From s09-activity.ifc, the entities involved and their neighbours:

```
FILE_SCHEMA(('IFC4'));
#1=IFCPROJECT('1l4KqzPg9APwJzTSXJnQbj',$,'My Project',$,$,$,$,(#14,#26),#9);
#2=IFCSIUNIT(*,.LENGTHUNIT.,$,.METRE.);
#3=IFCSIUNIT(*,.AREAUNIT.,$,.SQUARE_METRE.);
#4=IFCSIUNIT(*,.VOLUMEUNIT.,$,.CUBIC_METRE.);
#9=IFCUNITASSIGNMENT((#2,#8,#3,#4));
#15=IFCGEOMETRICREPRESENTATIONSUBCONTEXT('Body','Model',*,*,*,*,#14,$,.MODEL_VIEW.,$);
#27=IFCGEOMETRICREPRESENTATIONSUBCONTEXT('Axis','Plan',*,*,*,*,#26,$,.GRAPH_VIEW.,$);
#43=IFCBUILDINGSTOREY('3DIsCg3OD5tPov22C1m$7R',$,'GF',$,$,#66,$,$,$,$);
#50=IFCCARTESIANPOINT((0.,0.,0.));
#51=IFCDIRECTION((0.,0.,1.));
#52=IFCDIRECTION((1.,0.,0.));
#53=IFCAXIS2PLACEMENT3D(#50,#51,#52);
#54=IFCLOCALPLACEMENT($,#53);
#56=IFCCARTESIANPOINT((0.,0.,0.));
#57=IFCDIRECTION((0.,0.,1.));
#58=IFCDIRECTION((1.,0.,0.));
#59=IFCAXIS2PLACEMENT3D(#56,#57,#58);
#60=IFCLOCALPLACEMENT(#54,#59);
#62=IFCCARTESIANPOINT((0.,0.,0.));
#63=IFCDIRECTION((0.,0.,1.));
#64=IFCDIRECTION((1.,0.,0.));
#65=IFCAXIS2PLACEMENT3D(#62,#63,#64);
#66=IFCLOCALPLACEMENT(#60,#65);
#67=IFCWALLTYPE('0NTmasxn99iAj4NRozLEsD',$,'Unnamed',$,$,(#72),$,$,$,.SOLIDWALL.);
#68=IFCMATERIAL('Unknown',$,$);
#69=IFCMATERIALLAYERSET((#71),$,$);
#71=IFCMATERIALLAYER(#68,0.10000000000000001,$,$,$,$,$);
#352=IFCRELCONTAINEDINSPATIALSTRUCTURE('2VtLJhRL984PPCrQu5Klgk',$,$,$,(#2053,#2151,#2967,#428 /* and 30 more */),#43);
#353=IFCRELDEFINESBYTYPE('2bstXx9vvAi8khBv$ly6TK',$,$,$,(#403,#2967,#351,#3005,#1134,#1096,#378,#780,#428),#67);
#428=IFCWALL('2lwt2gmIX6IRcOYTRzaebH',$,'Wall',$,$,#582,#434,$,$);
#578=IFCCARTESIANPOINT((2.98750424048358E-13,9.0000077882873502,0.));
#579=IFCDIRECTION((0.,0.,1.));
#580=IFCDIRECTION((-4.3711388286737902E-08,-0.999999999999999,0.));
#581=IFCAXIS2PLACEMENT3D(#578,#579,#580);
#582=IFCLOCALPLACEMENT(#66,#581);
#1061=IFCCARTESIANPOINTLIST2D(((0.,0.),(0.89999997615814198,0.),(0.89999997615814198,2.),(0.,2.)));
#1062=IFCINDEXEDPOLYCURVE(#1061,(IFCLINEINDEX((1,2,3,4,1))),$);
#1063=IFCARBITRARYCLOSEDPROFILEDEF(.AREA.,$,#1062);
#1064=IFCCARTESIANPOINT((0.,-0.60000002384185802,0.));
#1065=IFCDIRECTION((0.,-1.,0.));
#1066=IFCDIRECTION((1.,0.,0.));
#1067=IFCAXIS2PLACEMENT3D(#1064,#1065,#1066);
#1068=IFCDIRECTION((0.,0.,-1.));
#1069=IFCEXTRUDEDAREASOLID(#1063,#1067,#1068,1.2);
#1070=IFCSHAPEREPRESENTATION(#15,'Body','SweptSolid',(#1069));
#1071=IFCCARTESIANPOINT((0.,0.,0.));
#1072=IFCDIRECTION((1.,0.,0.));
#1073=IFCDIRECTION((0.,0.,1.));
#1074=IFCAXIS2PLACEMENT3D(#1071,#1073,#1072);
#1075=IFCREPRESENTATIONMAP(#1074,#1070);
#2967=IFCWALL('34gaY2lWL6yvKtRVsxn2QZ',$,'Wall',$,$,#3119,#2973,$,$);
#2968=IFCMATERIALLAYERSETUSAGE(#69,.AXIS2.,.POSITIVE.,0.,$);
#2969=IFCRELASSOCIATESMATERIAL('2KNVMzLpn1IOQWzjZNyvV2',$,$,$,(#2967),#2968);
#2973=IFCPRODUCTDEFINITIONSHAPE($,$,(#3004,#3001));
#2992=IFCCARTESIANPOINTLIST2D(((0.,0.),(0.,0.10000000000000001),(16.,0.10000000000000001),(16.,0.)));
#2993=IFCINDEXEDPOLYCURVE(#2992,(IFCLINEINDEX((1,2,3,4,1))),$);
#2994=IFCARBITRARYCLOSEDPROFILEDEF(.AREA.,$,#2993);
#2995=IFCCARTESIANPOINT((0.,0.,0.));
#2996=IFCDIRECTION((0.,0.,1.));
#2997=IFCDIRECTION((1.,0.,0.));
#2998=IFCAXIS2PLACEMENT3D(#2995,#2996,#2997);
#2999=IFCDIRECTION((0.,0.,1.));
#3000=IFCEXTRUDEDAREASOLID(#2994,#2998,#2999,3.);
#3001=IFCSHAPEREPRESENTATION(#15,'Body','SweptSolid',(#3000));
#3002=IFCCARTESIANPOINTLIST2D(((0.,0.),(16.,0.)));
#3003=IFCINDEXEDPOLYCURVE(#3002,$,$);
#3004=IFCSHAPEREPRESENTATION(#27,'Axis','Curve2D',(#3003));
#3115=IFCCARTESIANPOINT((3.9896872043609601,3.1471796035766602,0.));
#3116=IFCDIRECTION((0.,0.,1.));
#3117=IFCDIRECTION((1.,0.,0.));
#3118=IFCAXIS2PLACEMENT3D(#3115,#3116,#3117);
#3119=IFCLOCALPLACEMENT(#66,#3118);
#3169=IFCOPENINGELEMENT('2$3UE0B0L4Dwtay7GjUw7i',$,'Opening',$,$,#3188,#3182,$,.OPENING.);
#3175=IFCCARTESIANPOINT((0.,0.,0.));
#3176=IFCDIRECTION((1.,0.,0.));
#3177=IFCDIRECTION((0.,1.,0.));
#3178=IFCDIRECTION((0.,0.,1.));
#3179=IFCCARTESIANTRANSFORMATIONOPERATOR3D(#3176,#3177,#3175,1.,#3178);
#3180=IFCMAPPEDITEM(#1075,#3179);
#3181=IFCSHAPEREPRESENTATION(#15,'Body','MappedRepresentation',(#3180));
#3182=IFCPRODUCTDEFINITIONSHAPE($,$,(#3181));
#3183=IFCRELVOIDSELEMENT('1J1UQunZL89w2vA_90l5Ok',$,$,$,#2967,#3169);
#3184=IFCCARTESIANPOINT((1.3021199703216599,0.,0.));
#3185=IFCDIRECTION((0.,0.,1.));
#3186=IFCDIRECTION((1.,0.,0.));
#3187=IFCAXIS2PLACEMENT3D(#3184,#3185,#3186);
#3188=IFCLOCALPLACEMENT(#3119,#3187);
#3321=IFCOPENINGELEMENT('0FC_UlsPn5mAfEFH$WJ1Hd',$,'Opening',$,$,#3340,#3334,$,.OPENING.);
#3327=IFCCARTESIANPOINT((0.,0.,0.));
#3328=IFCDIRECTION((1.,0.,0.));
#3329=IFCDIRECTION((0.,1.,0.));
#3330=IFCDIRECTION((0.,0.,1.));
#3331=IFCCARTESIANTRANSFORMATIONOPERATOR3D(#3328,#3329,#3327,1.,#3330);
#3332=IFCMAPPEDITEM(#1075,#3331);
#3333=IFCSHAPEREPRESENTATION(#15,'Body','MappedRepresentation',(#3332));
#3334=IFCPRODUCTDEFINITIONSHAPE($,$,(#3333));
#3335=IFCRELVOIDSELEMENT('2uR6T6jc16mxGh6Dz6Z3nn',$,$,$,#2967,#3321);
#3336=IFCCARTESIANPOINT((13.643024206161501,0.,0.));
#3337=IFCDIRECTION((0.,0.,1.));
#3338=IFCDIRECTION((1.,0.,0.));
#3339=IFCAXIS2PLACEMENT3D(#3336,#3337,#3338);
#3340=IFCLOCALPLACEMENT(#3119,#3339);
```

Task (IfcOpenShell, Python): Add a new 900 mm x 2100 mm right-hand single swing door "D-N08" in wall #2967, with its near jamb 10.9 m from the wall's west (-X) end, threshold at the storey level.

```python
import numpy as np
import ifcopenshell
import ifcopenshell.api.feature
import ifcopenshell.api.geometry
import ifcopenshell.api.root
import ifcopenshell.api.spatial
import ifcopenshell.geom
import ifcopenshell.util.element
import ifcopenshell.util.placement
import ifcopenshell.util.representation
import ifcopenshell.util.shape
import ifcopenshell.util.unit

model = ifcopenshell.open("s09-activity.ifc")
unit_scale = ifcopenshell.util.unit.calculate_unit_scale(model)
settings = ifcopenshell.geom.settings()


def volume(element):
    """Net volume in cubic metres, openings subtracted."""
    shape = ifcopenshell.geom.create_shape(settings, element)
    return ifcopenshell.util.shape.get_volume(shape.geometry)


wall = model.by_id(2967)
storey = ifcopenshell.util.element.get_container(wall, ifc_class="IfcBuildingStorey")
context = ifcopenshell.util.representation.get_context(model, "Model", "Body", "MODEL_VIEW")
before = volume(wall)

width, height, from_end, sill = 0.9, 2.1, 10.9, 0.0  # metres

# The wall runs along its own X axis, and the end named is its -X end.
wall_shape = ifcopenshell.geom.create_shape(settings, wall)
x, y, z = ifcopenshell.util.shape.get_vertices(wall_shape.geometry).T
start = x.min() + from_end
face, thickness = float(y.min()), float(y.max() - y.min())
wall_matrix = ifcopenshell.util.placement.get_local_placement(wall.ObjectPlacement)
level = ifcopenshell.util.placement.get_local_placement(storey.ObjectPlacement)[2, 3]


def in_wall(x, y):
    """Placement at x, y metres in the wall's axes, at sill height."""
    matrix = wall_matrix.copy()
    matrix[:, 3] = wall_matrix @ np.array([x / unit_scale, y / unit_scale, 0.0, 1.0])
    matrix[2, 3] = level + sill / unit_scale
    return matrix


# Opening: a box that overshoots both wall faces by 50 mm.
opening = ifcopenshell.api.root.create_entity(model, ifc_class="IfcOpeningElement", predefined_type="OPENING")
box = ifcopenshell.api.geometry.add_wall_representation(
    model, context=context, length=width, height=height, thickness=thickness + 0.1
)
ifcopenshell.api.geometry.assign_representation(model, product=opening, representation=box)
ifcopenshell.api.geometry.edit_object_placement(model, product=opening, matrix=in_wall(start, face - 0.05), is_si=False)
ifcopenshell.api.feature.add_feature(model, feature=opening, element=wall)

door = ifcopenshell.api.root.create_entity(model, ifc_class="IfcDoor", name="D-N08", predefined_type="DOOR")
door.OverallWidth, door.OverallHeight = width / unit_scale, height / unit_scale
door.OperationType = "SINGLE_SWING_RIGHT"
body = ifcopenshell.api.geometry.add_door_representation(
    model,
    context=context,
    overall_width=door.OverallWidth,
    overall_height=door.OverallHeight,
    operation_type="SINGLE_SWING_RIGHT",
    lining_properties={"LiningDepth": thickness / unit_scale, "ThresholdDepth": thickness / unit_scale},
)
ifcopenshell.api.geometry.assign_representation(model, product=door, representation=body)
ifcopenshell.api.spatial.assign_container(model, products=[door], relating_structure=storey)
ifcopenshell.api.feature.add_filling(model, opening=opening, element=door)

# The lining spans the wall, so the door starts at the wall face.
ifcopenshell.api.geometry.edit_object_placement(model, product=door, matrix=in_wall(start, face), is_si=False)

after = volume(wall)

print(f"wall volume {before:.3f} -> {after:.3f} m3")

model.write("s09-activity-out.ifc")
```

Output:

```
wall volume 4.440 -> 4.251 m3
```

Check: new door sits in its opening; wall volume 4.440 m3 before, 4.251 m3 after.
